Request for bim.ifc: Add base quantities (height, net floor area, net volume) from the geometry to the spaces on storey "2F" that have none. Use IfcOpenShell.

First a look at what the model holds.

```python
import ifcopenshell
import ifcopenshell.util.element
import ifcopenshell.util.unit

model = ifcopenshell.open("bim.ifc")
print(model.schema)
for unit_type in ("LENGTHUNIT", "AREAUNIT", "VOLUMEUNIT"):
    print(unit_type, ifcopenshell.util.unit.calculate_unit_scale(model, unit_type))
storey = next(s for s in model.by_type("IfcBuildingStorey") if s.Name == "2F")
spaces = [e for e in ifcopenshell.util.element.get_decomposition(storey) if e.is_a("IfcSpace")]
for e in sorted(spaces, key=lambda e: e.id()):
    print(e.id(), e.is_a(), e.Name, list(ifcopenshell.util.element.get_psets(e, qtos_only=True)), sep=" | ")
```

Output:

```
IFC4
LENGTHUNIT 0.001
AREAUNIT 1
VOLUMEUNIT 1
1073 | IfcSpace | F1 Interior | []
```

```python
import ifcopenshell
import ifcopenshell.api.pset
import ifcopenshell.geom
import ifcopenshell.util.element
import ifcopenshell.util.shape
import ifcopenshell.util.unit

model = ifcopenshell.open("bim.ifc")
unit_scale = ifcopenshell.util.unit.calculate_unit_scale(model)
area_scale = ifcopenshell.util.unit.calculate_unit_scale(model, "AREAUNIT")
volume_scale = ifcopenshell.util.unit.calculate_unit_scale(model, "VOLUMEUNIT")
settings = ifcopenshell.geom.settings()

storey = next(s for s in model.by_type("IfcBuildingStorey") if s.Name == "2F")
spaces = [e for e in ifcopenshell.util.element.get_decomposition(storey) if e.is_a("IfcSpace")]

for e in sorted(spaces, key=lambda e: e.id()):
    if ifcopenshell.util.element.get_psets(e, qtos_only=True, should_inherit=False):
        continue
    # Geometry comes back in metres, in the element's own axes.
    shape = ifcopenshell.geom.create_shape(settings, e)
    values = {
        "Height": ifcopenshell.util.shape.get_z(shape.geometry) / unit_scale,
        "NetFloorArea": ifcopenshell.util.shape.get_footprint_area(shape.geometry) / area_scale,
        "NetVolume": ifcopenshell.util.shape.get_volume(shape.geometry) / volume_scale,
    }
    qto = ifcopenshell.api.pset.add_qto(model, product=e, name="Qto_SpaceBaseQuantities")
    ifcopenshell.api.pset.edit_qto(model, qto=qto, properties=values)
    print(e.id(), {k: round(v, 3) for k, v in values.items()})

model.write("bim_edited.ifc")
```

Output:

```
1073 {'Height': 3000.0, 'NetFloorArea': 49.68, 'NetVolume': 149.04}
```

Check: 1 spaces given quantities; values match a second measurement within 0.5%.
